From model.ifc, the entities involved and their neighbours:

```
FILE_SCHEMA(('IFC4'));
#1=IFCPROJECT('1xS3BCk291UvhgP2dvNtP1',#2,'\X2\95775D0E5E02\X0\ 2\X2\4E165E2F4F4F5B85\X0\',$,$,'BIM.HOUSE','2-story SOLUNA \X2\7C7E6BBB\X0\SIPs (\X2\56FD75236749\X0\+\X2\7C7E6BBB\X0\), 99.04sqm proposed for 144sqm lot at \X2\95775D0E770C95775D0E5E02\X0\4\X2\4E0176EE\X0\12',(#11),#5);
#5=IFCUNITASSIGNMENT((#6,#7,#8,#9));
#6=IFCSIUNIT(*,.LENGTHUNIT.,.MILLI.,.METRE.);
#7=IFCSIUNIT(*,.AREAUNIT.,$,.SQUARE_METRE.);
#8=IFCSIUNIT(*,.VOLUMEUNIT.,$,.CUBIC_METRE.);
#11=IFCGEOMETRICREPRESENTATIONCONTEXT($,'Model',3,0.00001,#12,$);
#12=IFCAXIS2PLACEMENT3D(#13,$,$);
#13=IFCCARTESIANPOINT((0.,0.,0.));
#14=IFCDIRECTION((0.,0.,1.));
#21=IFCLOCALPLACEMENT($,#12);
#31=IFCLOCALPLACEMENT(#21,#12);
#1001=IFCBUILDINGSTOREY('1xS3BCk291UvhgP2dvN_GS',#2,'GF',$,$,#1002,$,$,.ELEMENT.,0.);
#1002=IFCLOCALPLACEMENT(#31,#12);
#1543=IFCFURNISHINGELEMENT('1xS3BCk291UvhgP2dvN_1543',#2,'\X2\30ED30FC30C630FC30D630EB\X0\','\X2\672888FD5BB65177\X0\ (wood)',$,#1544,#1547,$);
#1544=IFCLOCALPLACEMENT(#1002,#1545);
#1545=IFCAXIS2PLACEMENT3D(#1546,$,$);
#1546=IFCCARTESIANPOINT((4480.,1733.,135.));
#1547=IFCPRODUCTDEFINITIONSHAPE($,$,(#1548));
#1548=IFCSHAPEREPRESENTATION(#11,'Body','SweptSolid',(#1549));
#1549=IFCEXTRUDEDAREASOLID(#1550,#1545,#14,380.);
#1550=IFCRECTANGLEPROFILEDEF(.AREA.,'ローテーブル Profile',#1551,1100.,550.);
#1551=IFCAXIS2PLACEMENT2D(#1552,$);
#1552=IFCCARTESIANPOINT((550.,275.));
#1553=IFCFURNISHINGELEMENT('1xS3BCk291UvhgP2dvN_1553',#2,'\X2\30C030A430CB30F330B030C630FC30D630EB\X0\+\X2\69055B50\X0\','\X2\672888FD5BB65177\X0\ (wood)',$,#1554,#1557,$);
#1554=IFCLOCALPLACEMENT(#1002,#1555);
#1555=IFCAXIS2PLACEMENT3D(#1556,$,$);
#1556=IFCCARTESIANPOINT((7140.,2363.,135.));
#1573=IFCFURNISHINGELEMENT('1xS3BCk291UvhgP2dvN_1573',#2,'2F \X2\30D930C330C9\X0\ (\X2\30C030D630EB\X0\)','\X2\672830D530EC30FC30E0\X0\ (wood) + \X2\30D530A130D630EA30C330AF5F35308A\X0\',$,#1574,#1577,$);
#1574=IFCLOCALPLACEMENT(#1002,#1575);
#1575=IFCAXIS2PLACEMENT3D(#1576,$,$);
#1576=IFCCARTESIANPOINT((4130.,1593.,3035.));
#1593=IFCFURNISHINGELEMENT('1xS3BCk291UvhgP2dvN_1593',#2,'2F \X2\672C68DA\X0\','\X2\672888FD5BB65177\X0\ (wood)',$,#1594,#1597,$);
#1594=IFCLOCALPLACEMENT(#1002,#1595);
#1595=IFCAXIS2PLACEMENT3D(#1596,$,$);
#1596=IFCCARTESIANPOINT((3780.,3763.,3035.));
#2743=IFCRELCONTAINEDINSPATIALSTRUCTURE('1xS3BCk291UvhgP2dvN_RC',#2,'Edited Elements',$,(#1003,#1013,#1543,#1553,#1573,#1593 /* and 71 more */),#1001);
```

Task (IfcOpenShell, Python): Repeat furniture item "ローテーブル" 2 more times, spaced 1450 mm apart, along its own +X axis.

```python
import ifcopenshell
import ifcopenshell.api.geometry
import ifcopenshell.api.root
import ifcopenshell.util.element
import ifcopenshell.util.placement

model = ifcopenshell.open("model.ifc")


def reuse_history(source, copy):
    """copy_class also copies each property set's owner history, people and application; keep the originals."""
    for rel in copy.IsDefinedBy:
        if rel.is_a("IfcRelDefinesByProperties") and (history := rel.RelatingPropertyDefinition.OwnerHistory):
            rel.RelatingPropertyDefinition.OwnerHistory = source.OwnerHistory
            ifcopenshell.util.element.remove_deep2(model, history)


source = model.by_guid("1xS3BCk291UvhgP2dvN_1543")
base = ifcopenshell.util.placement.get_local_placement(source.ObjectPlacement)
step = base[:3, 0] * 1450.0

for i in range(1, 3):
    copy = ifcopenshell.api.root.copy_class(model, product=source)
    copy.Representation = ifcopenshell.util.element.copy_deep(
        model, source.Representation, exclude=["IfcGeometricRepresentationContext", "IfcRepresentationMap"]
    )
    reuse_history(source, copy)
    matrix = base.copy()
    matrix[:3, 3] += i * step
    print("added at", matrix[:3, 3].round(3) + 0.0)
    ifcopenshell.api.geometry.edit_object_placement(model, product=copy, matrix=matrix, is_si=False)

model.write("model_rev.ifc")
```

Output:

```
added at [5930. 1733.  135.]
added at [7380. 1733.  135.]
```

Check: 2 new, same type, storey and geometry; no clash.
